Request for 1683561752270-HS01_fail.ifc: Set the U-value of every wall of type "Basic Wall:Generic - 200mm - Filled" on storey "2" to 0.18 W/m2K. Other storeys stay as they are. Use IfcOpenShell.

First a look at what the model holds.

```python
import ifcopenshell
import ifcopenshell.util.element

model = ifcopenshell.open("1683561752270-HS01_fail.ifc")
print(model.schema)
storey = next(s for s in model.by_type("IfcBuildingStorey") if s.Name == "2")
walls = [e for e in ifcopenshell.util.element.get_decomposition(storey) if e.is_a("IfcWall")]
seen = {}
for e in walls:
    element_type = ifcopenshell.util.element.get_type(e)
    key = (element_type.Name if element_type != e and element_type else None, ifcopenshell.util.element.get_pset(e, "Pset_WallCommon", "ThermalTransmittance"))
    seen[key] = seen.get(key, 0) + 1
for (name, value), count in sorted(seen.items(), key=str):
    print(count, "x", name, "|", value)
```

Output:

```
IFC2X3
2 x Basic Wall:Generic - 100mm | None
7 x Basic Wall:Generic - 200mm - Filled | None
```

```python
import ifcopenshell
import ifcopenshell.api.pset
import ifcopenshell.util.element

model = ifcopenshell.open("1683561752270-HS01_fail.ifc")

storey = next(s for s in model.by_type("IfcBuildingStorey") if s.Name == "2")
walls = [e for e in ifcopenshell.util.element.get_decomposition(storey) if e.is_a("IfcWall")]

count = 0
for e in walls:
    element_type = ifcopenshell.util.element.get_type(e)
    if element_type in (None, e) or element_type.Name != "Basic Wall:Generic - 200mm - Filled":
        continue
    # add_pset returns the element's existing set when there is one.
    pset = ifcopenshell.api.pset.add_pset(model, product=e, name="Pset_WallCommon")
    ifcopenshell.api.pset.edit_pset(model, pset=pset, properties={"ThermalTransmittance": 0.18})
    count += 1

print(count, "walls updated")

model.write("1683561752270-HS01_fail_v2.ifc")
```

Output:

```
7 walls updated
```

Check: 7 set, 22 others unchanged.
